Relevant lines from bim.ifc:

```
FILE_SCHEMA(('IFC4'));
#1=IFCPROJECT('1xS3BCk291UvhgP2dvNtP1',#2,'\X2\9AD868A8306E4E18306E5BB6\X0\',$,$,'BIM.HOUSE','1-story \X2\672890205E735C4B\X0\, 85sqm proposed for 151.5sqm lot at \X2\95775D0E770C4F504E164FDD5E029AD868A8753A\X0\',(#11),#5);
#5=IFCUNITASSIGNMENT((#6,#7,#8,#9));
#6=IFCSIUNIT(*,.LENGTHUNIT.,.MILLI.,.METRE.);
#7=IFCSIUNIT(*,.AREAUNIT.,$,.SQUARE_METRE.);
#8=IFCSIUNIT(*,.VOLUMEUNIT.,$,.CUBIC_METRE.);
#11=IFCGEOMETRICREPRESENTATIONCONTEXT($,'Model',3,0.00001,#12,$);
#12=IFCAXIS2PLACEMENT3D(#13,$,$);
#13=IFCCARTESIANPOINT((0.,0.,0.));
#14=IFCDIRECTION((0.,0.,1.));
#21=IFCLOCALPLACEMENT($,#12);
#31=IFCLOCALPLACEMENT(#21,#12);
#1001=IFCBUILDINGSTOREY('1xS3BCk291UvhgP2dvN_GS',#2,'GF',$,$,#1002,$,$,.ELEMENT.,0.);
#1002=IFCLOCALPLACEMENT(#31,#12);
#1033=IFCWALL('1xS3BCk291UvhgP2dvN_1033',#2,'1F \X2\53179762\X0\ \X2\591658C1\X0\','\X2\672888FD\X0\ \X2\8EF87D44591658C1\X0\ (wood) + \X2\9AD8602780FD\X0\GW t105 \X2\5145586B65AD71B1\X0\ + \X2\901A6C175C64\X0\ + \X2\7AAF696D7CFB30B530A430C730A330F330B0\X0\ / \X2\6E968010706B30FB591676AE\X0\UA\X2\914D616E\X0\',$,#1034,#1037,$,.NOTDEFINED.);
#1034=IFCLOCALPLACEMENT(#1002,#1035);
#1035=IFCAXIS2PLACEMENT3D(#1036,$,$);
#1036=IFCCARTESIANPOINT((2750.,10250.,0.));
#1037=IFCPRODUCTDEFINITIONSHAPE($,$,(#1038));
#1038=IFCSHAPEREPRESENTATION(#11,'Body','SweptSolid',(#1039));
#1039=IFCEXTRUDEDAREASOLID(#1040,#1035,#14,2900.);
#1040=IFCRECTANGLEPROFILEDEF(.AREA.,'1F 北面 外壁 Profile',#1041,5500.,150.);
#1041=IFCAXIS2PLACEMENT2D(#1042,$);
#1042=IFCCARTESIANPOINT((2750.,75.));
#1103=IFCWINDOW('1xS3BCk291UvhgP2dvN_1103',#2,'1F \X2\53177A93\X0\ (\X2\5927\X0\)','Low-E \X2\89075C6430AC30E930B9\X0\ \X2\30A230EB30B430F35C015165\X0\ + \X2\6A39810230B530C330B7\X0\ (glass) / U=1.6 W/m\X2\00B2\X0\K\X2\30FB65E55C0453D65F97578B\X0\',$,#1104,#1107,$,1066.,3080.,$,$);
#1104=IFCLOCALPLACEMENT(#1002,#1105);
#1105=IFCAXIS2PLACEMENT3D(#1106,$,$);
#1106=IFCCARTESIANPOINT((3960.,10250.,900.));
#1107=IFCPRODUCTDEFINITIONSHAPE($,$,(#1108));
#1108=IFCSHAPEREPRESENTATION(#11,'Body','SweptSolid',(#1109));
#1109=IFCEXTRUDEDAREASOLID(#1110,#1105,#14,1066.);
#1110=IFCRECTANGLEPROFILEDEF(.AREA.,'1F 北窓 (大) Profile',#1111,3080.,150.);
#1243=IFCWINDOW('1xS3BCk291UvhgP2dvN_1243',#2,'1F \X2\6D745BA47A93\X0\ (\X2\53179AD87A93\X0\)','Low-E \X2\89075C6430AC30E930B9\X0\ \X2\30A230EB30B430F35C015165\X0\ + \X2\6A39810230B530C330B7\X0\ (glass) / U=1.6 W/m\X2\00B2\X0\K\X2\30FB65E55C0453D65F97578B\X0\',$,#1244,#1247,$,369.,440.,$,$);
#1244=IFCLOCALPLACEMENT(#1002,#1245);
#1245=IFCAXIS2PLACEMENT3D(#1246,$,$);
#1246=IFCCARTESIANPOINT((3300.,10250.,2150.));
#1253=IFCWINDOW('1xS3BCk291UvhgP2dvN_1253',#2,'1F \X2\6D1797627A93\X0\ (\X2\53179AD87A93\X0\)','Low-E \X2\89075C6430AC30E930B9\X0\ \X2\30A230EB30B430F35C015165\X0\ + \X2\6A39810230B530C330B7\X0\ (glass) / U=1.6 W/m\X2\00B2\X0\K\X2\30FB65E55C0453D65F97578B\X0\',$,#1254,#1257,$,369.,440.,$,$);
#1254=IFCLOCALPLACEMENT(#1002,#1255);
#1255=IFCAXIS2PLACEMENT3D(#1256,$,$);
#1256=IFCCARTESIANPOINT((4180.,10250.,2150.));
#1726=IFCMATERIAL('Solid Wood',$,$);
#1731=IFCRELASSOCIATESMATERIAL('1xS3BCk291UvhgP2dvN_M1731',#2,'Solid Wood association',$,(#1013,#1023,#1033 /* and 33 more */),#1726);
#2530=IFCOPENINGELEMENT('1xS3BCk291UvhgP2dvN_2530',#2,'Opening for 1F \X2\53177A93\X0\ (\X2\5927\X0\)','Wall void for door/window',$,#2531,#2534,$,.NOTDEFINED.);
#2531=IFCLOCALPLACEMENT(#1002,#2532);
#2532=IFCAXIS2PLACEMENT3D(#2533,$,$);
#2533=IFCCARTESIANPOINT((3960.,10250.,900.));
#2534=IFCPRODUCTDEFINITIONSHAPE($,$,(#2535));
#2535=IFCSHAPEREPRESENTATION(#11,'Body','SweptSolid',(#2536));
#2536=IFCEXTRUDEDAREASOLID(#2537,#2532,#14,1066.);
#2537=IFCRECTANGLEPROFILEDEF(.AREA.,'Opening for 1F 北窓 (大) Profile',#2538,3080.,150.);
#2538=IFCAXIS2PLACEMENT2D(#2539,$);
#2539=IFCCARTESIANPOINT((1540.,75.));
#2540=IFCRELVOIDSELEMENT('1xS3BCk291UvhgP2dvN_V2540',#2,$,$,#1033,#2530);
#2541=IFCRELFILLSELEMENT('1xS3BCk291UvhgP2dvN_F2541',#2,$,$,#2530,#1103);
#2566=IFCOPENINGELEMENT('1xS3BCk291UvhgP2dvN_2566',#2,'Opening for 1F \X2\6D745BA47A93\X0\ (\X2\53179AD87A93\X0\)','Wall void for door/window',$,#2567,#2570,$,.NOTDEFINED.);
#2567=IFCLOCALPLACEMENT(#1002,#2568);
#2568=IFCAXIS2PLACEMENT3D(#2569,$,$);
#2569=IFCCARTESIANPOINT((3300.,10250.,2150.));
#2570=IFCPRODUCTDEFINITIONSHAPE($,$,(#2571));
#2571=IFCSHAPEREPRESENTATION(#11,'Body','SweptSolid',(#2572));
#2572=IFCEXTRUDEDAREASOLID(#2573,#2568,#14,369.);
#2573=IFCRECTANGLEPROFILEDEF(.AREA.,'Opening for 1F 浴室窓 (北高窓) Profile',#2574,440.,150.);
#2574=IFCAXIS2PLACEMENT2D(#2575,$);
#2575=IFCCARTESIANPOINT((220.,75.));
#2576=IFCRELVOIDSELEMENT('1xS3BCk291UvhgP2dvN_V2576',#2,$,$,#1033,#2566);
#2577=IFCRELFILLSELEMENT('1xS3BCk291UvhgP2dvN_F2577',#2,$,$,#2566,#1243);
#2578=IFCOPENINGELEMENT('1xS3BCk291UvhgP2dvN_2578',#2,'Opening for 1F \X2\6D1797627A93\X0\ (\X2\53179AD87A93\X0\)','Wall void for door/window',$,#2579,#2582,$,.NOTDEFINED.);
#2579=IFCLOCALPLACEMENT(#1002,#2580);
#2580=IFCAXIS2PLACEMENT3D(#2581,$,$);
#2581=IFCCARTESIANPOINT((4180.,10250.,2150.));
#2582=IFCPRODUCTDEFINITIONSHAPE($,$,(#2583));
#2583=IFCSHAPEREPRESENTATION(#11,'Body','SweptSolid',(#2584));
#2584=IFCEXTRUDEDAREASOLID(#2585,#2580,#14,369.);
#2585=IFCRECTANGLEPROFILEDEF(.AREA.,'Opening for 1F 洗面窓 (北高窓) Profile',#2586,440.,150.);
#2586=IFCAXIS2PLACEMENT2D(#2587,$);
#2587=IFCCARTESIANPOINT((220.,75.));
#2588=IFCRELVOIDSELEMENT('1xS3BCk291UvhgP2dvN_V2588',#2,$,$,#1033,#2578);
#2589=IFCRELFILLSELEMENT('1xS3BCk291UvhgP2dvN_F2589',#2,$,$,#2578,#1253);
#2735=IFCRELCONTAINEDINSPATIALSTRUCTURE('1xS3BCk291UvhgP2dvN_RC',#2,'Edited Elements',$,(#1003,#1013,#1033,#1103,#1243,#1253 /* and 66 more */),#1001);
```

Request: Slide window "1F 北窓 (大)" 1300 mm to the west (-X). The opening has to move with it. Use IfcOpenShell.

```python
import ifcopenshell
import ifcopenshell.api.geometry
import ifcopenshell.util.placement

model = ifcopenshell.open("bim.ifc")

window = model.by_guid("1xS3BCk291UvhgP2dvN_1103")
opening = window.FillsVoids[0].RelatingOpeningElement
wall = opening.VoidsElements[0].RelatingBuildingElement

wall_matrix = ifcopenshell.util.placement.get_local_placement(wall.ObjectPlacement)
shift = wall_matrix[:3, 0] * -1300.0
before = ifcopenshell.util.placement.get_local_placement(window.ObjectPlacement)[:3, 3].copy()

# The window is not placed relative to its opening, so move both.
for product in (opening, window):
    matrix = ifcopenshell.util.placement.get_local_placement(product.ObjectPlacement)
    matrix[:3, 3] += shift
    ifcopenshell.api.geometry.edit_object_placement(model, product=product, matrix=matrix, is_si=False)

after = ifcopenshell.util.placement.get_local_placement(window.ObjectPlacement)[:3, 3]
print("window moved by", (after - before).round(3) + 0.0)

model.write("bim_updated.ifc")
```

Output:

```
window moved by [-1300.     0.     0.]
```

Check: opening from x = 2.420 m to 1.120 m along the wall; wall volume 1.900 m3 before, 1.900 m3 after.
